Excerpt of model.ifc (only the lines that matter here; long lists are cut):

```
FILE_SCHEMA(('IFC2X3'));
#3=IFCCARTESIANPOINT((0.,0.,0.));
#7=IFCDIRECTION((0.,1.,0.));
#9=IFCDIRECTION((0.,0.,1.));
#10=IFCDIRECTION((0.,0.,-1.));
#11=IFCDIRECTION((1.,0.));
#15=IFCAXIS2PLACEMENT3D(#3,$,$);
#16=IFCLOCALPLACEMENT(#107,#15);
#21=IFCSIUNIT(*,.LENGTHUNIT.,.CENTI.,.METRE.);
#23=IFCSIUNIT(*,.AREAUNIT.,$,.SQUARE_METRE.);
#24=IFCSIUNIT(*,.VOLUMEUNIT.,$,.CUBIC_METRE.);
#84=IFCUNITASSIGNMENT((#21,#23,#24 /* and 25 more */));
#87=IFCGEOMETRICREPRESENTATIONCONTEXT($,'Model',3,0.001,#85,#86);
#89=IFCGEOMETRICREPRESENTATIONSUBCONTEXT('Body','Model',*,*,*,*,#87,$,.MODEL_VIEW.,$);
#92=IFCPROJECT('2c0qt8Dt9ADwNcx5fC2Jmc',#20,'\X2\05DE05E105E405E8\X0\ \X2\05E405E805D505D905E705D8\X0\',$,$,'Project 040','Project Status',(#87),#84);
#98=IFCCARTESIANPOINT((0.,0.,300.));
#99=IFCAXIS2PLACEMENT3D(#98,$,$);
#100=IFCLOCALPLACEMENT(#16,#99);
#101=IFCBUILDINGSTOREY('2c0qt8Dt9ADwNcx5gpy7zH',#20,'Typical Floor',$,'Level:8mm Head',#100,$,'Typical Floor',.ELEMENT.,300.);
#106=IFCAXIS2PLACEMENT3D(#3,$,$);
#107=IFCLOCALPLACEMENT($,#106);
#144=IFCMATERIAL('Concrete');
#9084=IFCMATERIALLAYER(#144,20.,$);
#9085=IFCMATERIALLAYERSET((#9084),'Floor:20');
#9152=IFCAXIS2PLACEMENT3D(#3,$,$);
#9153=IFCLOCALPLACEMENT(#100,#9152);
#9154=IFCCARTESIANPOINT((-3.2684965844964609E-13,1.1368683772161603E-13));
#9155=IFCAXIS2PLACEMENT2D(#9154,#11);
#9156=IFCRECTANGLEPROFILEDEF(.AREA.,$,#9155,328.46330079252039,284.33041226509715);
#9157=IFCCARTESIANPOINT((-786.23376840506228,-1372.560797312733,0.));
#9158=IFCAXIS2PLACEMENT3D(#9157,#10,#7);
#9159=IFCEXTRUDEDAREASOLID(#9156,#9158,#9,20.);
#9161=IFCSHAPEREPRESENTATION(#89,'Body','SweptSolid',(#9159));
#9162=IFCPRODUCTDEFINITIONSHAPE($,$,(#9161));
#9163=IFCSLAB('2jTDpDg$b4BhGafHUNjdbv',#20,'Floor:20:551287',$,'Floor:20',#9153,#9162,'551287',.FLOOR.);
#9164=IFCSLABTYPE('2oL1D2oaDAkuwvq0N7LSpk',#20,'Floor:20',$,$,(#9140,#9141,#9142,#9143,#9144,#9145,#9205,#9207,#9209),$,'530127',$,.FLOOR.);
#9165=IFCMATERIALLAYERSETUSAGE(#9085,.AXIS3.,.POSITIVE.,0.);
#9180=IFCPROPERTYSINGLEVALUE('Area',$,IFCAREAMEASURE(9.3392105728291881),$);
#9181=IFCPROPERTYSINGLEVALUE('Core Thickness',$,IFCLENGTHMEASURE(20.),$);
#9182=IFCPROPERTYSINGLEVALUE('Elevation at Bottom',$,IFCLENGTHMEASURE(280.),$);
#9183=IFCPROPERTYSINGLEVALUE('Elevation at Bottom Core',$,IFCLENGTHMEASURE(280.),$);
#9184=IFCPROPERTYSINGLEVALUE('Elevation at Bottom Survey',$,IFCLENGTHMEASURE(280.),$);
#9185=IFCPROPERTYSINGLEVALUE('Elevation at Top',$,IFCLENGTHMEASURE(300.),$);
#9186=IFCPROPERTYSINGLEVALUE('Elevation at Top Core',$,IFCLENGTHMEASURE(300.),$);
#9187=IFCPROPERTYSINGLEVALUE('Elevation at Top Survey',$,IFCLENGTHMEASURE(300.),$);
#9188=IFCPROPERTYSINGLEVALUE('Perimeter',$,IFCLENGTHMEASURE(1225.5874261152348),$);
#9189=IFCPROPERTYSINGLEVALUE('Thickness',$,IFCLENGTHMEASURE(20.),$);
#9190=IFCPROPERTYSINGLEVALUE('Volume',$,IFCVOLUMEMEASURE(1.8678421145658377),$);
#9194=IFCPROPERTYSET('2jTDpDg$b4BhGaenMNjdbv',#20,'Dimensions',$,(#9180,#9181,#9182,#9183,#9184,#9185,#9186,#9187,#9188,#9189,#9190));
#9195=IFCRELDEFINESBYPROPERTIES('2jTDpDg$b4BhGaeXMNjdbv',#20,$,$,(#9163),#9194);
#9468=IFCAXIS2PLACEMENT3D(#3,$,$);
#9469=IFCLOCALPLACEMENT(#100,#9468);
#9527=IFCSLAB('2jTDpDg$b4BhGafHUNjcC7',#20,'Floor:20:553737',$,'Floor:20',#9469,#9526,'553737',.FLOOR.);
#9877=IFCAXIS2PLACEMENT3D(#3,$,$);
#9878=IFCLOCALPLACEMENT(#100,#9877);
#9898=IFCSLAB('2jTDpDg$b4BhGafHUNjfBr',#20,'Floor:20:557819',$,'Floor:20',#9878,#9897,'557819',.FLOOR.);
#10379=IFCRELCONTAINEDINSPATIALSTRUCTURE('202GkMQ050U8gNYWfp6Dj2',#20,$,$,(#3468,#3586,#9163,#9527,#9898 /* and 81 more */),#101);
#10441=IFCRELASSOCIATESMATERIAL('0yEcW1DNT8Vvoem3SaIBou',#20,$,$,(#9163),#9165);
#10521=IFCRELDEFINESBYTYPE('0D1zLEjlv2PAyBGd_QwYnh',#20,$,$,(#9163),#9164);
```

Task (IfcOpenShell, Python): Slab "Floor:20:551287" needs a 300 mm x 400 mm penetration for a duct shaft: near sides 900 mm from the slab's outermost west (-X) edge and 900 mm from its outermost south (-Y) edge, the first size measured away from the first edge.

```python
import numpy as np
import ifcopenshell
import ifcopenshell.api.feature
import ifcopenshell.api.geometry
import ifcopenshell.api.pset
import ifcopenshell.api.root
import ifcopenshell.geom
import ifcopenshell.util.element
import ifcopenshell.util.placement
import ifcopenshell.util.representation
import ifcopenshell.util.shape
import ifcopenshell.util.unit

model = ifcopenshell.open("model.ifc")
unit_scale = ifcopenshell.util.unit.calculate_unit_scale(model)
area_scale = ifcopenshell.util.unit.calculate_unit_scale(model, "AREAUNIT")
volume_scale = ifcopenshell.util.unit.calculate_unit_scale(model, "VOLUMEUNIT")
settings = ifcopenshell.geom.settings()


def volume(element):
    """Net volume in cubic metres, openings subtracted."""
    shape = ifcopenshell.geom.create_shape(settings, element)
    return ifcopenshell.util.shape.get_volume(shape.geometry)


slab = model.by_guid("2jTDpDg$b4BhGafHUNjdbv")
before = volume(slab)

# Extent in the slab's own axes, in metres. The edges named are its -X and -Y sides.
slab_shape = ifcopenshell.geom.create_shape(settings, slab)
vertices = ifcopenshell.util.shape.get_vertices(slab_shape.geometry)
x_min, y_min, bottom = vertices.min(axis=0)
top = vertices[:, 2].max()

opening = ifcopenshell.api.root.create_entity(model, ifc_class="IfcOpeningElement", name="Duct shaft opening")
context = ifcopenshell.util.representation.get_context(model, "Model", "Body", "MODEL_VIEW")
width, depth = 0.3, 0.4
outline = [(0.0, 0.0), (width, 0.0), (width, depth), (0.0, depth), (0.0, 0.0)]
# Overshoot both faces by 50 mm so the cut is clean.
shape = ifcopenshell.api.geometry.add_slab_representation(
    model, context=context, depth=top - bottom + 0.1, polyline=outline
)
ifcopenshell.api.geometry.assign_representation(model, product=opening, representation=shape)

matrix = ifcopenshell.util.placement.get_local_placement(slab.ObjectPlacement)
matrix[:, 3] = matrix @ np.append(np.array([x_min + 0.9, y_min + 0.9, bottom - 0.05]) / unit_scale, 1.0)
ifcopenshell.api.geometry.edit_object_placement(model, product=opening, matrix=matrix, is_si=False)
ifcopenshell.api.feature.add_feature(model, feature=opening, element=slab)

after = volume(slab)

# Update the slab's stored quantities.
pset = model.by_id(ifcopenshell.util.element.get_pset(slab, "Dimensions", should_inherit=False)["id"])
ifcopenshell.api.pset.edit_pset(model, pset=pset, properties={
    "Area": model.create_entity("IfcAreaMeasure", after / (top - bottom) / area_scale),
    "Volume": model.create_entity("IfcVolumeMeasure", after / volume_scale),
})

print(f"slab volume {before:.3f} -> {after:.3f} m3")

model.write("model-out.ifc")
```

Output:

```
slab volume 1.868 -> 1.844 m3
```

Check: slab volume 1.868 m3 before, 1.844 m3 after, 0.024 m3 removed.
